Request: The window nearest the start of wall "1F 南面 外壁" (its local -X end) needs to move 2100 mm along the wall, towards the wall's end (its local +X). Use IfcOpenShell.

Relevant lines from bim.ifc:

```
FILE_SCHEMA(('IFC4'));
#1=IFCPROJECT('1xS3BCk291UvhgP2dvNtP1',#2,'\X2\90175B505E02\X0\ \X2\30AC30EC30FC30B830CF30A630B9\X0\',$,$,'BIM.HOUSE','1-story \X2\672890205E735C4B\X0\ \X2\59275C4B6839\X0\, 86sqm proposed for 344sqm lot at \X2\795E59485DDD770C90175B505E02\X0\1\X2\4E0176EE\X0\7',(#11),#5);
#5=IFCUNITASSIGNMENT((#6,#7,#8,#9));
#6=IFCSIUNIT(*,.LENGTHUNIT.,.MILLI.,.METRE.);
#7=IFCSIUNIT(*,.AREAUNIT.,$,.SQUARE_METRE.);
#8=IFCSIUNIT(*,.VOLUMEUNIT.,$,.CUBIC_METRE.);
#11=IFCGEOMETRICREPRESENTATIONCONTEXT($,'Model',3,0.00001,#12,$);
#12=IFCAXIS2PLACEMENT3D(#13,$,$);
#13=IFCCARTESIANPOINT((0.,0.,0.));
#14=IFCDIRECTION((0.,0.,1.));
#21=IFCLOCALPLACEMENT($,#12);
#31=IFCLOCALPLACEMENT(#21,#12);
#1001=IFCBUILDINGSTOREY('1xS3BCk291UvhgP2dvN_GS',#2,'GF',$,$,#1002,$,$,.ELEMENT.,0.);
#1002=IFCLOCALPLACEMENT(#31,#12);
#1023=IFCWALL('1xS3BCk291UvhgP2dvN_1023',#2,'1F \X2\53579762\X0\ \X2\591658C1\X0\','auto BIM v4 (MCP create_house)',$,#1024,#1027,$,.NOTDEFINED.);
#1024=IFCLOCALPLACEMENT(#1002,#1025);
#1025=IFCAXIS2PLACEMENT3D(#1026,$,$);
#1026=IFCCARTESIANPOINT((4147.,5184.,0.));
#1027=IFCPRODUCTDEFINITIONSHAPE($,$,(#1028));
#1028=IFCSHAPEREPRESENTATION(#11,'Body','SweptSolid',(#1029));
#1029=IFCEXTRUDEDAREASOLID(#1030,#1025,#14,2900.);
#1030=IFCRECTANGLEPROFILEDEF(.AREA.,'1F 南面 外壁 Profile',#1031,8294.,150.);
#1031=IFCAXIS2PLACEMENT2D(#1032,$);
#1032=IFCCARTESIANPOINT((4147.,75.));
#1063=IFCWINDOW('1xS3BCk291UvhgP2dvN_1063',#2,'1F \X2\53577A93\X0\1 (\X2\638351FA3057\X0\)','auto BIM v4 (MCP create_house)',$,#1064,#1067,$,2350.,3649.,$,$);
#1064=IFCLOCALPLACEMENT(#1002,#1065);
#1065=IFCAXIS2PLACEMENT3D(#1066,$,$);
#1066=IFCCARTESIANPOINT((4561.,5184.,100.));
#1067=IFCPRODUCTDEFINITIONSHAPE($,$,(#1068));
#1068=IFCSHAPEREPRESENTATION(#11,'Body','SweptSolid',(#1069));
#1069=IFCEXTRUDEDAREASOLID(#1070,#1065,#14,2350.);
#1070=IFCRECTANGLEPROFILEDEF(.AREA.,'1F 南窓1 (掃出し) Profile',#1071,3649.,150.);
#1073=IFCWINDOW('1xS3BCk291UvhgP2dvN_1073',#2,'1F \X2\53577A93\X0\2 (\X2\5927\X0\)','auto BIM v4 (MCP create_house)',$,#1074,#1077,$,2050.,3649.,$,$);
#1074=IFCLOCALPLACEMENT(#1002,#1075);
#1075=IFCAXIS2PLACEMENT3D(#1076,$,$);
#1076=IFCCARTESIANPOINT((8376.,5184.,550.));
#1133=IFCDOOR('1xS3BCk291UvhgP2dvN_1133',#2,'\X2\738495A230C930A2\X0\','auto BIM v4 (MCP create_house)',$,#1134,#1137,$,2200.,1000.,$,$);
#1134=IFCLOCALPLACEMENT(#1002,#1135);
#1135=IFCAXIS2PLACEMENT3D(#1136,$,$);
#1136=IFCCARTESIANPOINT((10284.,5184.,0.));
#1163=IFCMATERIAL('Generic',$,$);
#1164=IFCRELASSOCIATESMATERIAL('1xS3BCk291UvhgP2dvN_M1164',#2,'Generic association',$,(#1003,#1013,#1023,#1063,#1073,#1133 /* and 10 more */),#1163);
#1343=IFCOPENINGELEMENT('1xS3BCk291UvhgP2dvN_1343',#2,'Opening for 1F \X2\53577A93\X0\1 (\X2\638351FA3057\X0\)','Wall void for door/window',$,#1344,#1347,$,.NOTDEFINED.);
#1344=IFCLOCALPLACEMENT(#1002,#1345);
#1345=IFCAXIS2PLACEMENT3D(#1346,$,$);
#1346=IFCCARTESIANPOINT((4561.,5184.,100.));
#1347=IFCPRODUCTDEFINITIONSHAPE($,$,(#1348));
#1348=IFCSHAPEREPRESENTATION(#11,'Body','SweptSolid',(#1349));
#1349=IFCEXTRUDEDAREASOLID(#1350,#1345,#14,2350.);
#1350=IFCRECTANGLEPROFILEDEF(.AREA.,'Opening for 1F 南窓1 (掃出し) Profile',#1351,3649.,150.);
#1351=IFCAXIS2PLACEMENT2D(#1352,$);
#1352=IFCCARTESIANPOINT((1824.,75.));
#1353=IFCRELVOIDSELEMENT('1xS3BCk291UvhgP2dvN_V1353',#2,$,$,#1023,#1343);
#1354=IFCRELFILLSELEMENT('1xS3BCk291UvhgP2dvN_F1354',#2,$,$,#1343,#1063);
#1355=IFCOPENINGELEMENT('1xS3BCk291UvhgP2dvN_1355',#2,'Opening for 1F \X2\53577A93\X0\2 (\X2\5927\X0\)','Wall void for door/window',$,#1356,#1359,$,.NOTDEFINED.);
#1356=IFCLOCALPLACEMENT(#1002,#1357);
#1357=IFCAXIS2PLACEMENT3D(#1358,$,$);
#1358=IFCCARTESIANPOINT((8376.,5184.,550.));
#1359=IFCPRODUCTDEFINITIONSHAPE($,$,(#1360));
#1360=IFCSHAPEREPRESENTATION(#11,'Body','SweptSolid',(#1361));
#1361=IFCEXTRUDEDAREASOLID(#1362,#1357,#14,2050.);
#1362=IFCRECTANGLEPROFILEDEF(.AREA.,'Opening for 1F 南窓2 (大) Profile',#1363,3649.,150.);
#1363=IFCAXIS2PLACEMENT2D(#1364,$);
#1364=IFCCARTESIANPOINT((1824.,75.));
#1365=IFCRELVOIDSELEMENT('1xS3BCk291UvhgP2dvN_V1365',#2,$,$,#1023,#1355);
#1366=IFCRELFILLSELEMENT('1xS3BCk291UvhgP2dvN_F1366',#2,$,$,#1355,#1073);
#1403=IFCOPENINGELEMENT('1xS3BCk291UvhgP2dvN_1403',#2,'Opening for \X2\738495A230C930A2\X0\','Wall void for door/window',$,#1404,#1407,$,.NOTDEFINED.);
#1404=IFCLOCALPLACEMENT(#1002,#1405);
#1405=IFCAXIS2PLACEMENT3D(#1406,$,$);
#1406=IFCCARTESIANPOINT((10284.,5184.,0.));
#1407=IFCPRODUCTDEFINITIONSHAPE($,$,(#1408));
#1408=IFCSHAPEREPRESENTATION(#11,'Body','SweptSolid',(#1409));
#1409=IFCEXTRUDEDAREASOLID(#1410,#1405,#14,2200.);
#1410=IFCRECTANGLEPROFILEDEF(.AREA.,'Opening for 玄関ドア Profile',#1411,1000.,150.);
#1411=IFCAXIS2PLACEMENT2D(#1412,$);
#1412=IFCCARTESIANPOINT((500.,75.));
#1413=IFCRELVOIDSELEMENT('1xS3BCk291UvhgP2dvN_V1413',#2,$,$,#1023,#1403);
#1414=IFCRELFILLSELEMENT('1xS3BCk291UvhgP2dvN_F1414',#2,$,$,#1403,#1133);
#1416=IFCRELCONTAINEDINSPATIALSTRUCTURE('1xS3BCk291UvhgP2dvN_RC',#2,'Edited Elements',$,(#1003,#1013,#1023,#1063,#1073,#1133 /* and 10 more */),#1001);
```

```python
import ifcopenshell
import ifcopenshell.api.geometry
import ifcopenshell.util.placement
import ifcopenshell.util.unit

model = ifcopenshell.open("bim.ifc")
unit_scale = ifcopenshell.util.unit.calculate_unit_scale(model)

window = model.by_id(1063)
opening = window.FillsVoids[0].RelatingOpeningElement
wall = opening.VoidsElements[0].RelatingBuildingElement

wall_matrix = ifcopenshell.util.placement.get_local_placement(wall.ObjectPlacement)
shift = wall_matrix[:3, 0] * 2.1 / unit_scale
before = ifcopenshell.util.placement.get_local_placement(window.ObjectPlacement)[:3, 3].copy()

# The window is not placed relative to its opening, so move both.
for product in (opening, window):
    matrix = ifcopenshell.util.placement.get_local_placement(product.ObjectPlacement)
    matrix[:3, 3] += shift
    ifcopenshell.api.geometry.edit_object_placement(model, product=product, matrix=matrix, is_si=False)

after = ifcopenshell.util.placement.get_local_placement(window.ObjectPlacement)[:3, 3]
print("window moved by", (after - before).round(3) + 0.0)

model.write("bim-out.ifc")
```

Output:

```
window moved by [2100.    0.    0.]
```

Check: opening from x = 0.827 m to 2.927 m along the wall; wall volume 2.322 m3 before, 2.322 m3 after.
